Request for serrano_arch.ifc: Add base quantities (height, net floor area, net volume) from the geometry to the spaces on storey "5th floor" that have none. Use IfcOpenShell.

First a look at what the model holds.

```python
import ifcopenshell
import ifcopenshell.util.element
import ifcopenshell.util.unit

model = ifcopenshell.open("serrano_arch.ifc")
print(model.schema)
for unit_type in ("LENGTHUNIT", "AREAUNIT", "VOLUMEUNIT"):
    print(unit_type, ifcopenshell.util.unit.calculate_unit_scale(model, unit_type))
storey = next(s for s in model.by_type("IfcBuildingStorey") if s.Name == "5th floor")
spaces = [e for e in ifcopenshell.util.element.get_decomposition(storey) if e.is_a("IfcSpace")]
for e in sorted(spaces, key=lambda e: e.id()):
    print(e.id(), e.is_a(), e.Name, list(ifcopenshell.util.element.get_psets(e, qtos_only=True)), sep=" | ")
```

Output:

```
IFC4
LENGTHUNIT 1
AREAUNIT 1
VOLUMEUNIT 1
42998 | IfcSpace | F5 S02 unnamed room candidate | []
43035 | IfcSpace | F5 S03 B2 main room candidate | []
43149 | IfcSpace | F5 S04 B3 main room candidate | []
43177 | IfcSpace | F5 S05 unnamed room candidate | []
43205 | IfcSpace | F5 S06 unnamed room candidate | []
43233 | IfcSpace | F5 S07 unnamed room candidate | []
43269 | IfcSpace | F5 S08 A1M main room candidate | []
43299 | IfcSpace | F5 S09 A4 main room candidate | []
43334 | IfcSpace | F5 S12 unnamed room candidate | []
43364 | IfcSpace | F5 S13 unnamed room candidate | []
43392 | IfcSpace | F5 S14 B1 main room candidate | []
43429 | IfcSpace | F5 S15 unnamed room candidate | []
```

```python
import ifcopenshell
import ifcopenshell.api.pset
import ifcopenshell.geom
import ifcopenshell.util.element
import ifcopenshell.util.shape
import ifcopenshell.util.unit

model = ifcopenshell.open("serrano_arch.ifc")
unit_scale = ifcopenshell.util.unit.calculate_unit_scale(model)
area_scale = ifcopenshell.util.unit.calculate_unit_scale(model, "AREAUNIT")
volume_scale = ifcopenshell.util.unit.calculate_unit_scale(model, "VOLUMEUNIT")
settings = ifcopenshell.geom.settings()

storey = next(s for s in model.by_type("IfcBuildingStorey") if s.Name == "5th floor")
spaces = [e for e in ifcopenshell.util.element.get_decomposition(storey) if e.is_a("IfcSpace")]

for e in sorted(spaces, key=lambda e: e.id()):
    if ifcopenshell.util.element.get_psets(e, qtos_only=True, should_inherit=False):
        continue
    # Geometry comes back in metres, in the element's own axes.
    shape = ifcopenshell.geom.create_shape(settings, e)
    values = {
        "Height": ifcopenshell.util.shape.get_z(shape.geometry) / unit_scale,
        "NetFloorArea": ifcopenshell.util.shape.get_footprint_area(shape.geometry) / area_scale,
        "NetVolume": ifcopenshell.util.shape.get_volume(shape.geometry) / volume_scale,
    }
    qto = ifcopenshell.api.pset.add_qto(model, product=e, name="Qto_SpaceBaseQuantities")
    ifcopenshell.api.pset.edit_qto(model, qto=qto, properties=values)
    print(e.id(), {k: round(v, 3) for k, v in values.items()})

model.write("serrano_arch_rev.ifc")
```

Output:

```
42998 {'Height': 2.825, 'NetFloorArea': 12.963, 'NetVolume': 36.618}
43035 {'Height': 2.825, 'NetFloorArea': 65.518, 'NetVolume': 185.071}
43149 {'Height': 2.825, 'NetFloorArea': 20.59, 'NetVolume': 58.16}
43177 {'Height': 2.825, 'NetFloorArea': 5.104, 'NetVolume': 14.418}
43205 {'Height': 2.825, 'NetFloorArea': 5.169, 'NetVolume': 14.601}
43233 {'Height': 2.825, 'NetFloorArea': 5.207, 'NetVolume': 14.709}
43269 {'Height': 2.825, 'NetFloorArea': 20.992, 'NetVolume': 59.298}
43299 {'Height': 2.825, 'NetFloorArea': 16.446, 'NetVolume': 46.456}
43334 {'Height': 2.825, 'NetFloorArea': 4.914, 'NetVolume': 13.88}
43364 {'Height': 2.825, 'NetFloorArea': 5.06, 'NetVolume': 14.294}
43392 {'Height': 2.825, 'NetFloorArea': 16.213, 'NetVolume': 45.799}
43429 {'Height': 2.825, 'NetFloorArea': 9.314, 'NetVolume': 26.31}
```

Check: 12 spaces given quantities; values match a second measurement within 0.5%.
